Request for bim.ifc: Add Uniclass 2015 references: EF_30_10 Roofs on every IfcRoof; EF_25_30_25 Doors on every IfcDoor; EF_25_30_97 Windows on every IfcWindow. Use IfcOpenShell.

First a look at what the model holds.

```python
import ifcopenshell

model = ifcopenshell.open("bim.ifc")
print(model.schema)
print("classifications:", [c.Name for c in model.by_type("IfcClassification")])
for ifc_class in ("IfcDoor", "IfcRoof", "IfcStair", "IfcWall", "IfcWindow"):
    print(ifc_class, len(model.by_type(ifc_class)))
```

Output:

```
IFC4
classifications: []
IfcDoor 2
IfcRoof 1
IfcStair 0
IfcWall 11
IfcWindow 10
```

```python
import ifcopenshell
import ifcopenshell.api.classification

model = ifcopenshell.open("bim.ifc")

system = ifcopenshell.api.classification.add_classification(model, classification="Uniclass 2015")

codes = {
    "IfcRoof": ("EF_30_10", "Roofs"),
    "IfcDoor": ("EF_25_30_25", "Doors"),
    "IfcWindow": ("EF_25_30_97", "Windows"),
}
for ifc_class, (code, name) in codes.items():
    products = model.by_type(ifc_class)
    ifcopenshell.api.classification.add_reference(
        model, products=products, classification=system, identification=code, name=name
    )
    print(code, len(products))

model.write("bim_edited.ifc")
```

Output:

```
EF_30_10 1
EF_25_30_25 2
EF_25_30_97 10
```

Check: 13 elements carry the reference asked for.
